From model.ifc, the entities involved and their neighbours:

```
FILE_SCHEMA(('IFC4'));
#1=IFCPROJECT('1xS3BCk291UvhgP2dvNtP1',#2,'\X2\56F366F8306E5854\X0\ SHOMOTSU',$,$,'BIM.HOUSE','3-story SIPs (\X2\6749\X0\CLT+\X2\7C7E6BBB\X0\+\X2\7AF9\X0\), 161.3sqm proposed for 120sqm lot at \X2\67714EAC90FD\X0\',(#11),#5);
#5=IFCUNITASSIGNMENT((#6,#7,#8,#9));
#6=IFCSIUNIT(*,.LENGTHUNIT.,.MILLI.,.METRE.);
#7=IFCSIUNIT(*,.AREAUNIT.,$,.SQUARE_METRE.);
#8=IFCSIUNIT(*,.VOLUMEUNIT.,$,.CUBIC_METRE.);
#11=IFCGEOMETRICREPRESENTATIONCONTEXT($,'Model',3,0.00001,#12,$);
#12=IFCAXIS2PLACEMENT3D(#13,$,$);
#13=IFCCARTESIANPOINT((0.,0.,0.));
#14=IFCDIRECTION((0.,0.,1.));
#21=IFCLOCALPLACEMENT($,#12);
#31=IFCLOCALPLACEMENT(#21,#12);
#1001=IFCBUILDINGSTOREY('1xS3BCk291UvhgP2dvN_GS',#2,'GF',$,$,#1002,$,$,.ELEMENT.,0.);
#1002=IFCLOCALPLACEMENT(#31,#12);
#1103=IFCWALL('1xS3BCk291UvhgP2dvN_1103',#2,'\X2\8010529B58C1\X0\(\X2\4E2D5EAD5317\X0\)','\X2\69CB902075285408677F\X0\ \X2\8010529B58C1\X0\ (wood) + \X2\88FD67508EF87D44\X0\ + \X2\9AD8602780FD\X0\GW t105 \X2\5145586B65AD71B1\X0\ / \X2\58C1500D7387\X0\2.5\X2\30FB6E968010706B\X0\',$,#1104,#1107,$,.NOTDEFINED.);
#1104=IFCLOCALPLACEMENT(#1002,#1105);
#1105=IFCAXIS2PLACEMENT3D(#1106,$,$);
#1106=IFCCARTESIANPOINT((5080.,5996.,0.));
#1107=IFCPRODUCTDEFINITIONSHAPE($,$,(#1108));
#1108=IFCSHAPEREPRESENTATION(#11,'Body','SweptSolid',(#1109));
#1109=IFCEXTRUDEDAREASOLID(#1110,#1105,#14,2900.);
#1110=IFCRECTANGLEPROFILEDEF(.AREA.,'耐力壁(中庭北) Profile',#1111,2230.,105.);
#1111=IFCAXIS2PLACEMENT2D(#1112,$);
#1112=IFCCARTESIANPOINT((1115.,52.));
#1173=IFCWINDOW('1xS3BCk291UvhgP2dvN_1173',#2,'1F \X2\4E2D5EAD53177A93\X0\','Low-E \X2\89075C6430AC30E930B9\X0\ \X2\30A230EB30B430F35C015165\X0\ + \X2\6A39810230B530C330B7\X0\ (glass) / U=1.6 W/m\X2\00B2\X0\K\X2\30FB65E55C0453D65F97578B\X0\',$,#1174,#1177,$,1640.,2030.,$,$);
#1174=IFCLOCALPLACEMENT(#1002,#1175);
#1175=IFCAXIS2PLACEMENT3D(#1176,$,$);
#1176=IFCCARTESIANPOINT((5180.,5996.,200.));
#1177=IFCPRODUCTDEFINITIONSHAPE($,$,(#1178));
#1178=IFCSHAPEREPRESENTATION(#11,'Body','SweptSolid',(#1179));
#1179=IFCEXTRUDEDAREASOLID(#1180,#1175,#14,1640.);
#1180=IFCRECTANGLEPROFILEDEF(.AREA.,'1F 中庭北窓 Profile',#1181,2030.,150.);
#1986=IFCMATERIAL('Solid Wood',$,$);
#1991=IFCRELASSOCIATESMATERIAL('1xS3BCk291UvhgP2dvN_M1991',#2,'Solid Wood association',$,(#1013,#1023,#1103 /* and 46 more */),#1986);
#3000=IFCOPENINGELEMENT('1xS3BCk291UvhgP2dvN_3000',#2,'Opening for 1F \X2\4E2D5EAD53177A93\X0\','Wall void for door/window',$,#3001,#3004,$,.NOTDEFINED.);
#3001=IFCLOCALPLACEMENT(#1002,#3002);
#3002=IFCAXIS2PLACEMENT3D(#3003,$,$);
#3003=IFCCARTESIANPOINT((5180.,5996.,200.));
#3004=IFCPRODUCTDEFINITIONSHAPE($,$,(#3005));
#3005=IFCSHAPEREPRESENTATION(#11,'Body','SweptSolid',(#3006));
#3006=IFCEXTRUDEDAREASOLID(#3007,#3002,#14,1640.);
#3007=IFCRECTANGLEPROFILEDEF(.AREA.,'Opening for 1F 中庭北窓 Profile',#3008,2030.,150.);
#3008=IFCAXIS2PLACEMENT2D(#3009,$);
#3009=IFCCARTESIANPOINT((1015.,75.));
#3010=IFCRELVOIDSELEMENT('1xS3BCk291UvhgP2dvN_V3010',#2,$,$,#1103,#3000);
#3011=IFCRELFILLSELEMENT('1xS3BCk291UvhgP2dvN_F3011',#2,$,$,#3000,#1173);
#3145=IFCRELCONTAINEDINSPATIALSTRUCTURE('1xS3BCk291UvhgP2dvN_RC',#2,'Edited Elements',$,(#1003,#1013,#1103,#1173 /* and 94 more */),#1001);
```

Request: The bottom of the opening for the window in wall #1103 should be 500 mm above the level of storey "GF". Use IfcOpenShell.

```python
import numpy as np
import ifcopenshell
import ifcopenshell.api.geometry
import ifcopenshell.geom
import ifcopenshell.util.element
import ifcopenshell.util.placement
import ifcopenshell.util.shape
import ifcopenshell.util.unit

model = ifcopenshell.open("model.ifc")
unit_scale = ifcopenshell.util.unit.calculate_unit_scale(model)

window = model.by_guid("1xS3BCk291UvhgP2dvN_1173")
opening = window.FillsVoids[0].RelatingOpeningElement
storey = ifcopenshell.util.element.get_container(window, ifc_class="IfcBuildingStorey")
level = ifcopenshell.util.placement.get_local_placement(storey.ObjectPlacement)[2, 3]

# The opening's origin need not be at the sill, so measure its lowest point.
shape = ifcopenshell.geom.create_shape(ifcopenshell.geom.settings(), opening)
bottom = ifcopenshell.util.shape.get_shape_bottom_elevation(shape, shape.geometry) / unit_scale
dz = level + 0.5 / unit_scale - bottom

shift = np.array([0.0, 0.0, dz])
# The window is not placed relative to its opening, so move both.
for product in (opening, window):
    matrix = ifcopenshell.util.placement.get_local_placement(product.ObjectPlacement)
    matrix[:3, 3] += shift
    ifcopenshell.api.geometry.edit_object_placement(model, product=product, matrix=matrix, is_si=False)

print(f"moved by {dz * unit_scale:+.3f} m")

model.write("model_edited.ifc")
```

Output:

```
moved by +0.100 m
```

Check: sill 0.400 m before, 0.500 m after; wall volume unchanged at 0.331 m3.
